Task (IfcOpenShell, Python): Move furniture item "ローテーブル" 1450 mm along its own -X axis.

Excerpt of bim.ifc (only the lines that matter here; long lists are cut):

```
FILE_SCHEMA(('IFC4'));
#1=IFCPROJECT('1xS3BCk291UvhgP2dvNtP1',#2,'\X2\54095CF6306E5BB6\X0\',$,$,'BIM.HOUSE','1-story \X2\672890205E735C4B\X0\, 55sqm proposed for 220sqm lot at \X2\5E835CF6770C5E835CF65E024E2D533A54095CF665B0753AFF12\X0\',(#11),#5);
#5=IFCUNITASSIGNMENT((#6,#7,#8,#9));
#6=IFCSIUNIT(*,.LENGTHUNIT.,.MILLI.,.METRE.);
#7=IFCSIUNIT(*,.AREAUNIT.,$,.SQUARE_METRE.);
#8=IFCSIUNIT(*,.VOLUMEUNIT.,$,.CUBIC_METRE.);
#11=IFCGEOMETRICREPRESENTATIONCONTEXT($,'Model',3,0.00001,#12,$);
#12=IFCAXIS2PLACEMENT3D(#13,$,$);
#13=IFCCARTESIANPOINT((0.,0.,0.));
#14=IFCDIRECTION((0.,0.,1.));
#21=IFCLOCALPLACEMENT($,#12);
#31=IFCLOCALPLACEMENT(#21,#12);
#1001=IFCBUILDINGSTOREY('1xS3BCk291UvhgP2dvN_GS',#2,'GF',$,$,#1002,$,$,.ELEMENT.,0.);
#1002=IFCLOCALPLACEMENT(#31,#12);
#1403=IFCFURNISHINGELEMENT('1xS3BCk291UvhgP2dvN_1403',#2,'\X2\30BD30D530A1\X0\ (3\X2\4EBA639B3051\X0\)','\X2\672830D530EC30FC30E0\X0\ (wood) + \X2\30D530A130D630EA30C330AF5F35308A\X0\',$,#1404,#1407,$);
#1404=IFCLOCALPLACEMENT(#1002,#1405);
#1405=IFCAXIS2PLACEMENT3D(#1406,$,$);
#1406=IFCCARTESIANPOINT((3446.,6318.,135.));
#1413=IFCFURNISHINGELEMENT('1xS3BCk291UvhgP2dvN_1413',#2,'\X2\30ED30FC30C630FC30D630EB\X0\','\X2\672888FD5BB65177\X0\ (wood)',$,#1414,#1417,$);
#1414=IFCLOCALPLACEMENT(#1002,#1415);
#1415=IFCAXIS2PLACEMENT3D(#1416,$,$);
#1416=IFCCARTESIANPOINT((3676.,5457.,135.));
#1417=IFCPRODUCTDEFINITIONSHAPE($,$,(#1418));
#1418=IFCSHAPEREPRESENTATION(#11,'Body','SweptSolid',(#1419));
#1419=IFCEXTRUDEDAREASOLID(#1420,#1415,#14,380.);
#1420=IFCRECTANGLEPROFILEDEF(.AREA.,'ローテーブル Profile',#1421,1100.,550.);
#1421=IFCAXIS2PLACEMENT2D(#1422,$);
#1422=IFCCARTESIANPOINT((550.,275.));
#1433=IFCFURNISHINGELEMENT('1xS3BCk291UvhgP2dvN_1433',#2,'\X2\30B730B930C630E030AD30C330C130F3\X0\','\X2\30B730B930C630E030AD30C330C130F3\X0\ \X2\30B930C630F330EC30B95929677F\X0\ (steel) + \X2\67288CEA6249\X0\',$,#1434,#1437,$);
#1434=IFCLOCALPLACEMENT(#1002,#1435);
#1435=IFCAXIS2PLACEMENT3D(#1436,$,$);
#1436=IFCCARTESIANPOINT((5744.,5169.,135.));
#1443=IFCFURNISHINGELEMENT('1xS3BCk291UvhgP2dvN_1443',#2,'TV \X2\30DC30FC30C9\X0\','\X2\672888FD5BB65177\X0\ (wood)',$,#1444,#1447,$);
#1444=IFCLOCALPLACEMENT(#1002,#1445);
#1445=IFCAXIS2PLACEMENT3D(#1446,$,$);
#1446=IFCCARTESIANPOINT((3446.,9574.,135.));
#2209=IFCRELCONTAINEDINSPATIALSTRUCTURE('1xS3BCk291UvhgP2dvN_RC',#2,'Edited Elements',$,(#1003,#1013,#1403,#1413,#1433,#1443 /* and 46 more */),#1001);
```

```python
import ifcopenshell
import ifcopenshell.api.geometry
import ifcopenshell.util.placement
import ifcopenshell.util.unit

model = ifcopenshell.open("bim.ifc")
unit_scale = ifcopenshell.util.unit.calculate_unit_scale(model)

item = model.by_guid("1xS3BCk291UvhgP2dvN_1413")
matrix = ifcopenshell.util.placement.get_local_placement(item.ObjectPlacement)
matrix[:3, 3] -= matrix[:3, 0] * 1.45 / unit_scale
ifcopenshell.api.geometry.edit_object_placement(model, product=item, matrix=matrix, is_si=False)

print(ifcopenshell.util.placement.get_local_placement(item.ObjectPlacement).round(3) + 0.0)

model.write("bim_v2.ifc")
```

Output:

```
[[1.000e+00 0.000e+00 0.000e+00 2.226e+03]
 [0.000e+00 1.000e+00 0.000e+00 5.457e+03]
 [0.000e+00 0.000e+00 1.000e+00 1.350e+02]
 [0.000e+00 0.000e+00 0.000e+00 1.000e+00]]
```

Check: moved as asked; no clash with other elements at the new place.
